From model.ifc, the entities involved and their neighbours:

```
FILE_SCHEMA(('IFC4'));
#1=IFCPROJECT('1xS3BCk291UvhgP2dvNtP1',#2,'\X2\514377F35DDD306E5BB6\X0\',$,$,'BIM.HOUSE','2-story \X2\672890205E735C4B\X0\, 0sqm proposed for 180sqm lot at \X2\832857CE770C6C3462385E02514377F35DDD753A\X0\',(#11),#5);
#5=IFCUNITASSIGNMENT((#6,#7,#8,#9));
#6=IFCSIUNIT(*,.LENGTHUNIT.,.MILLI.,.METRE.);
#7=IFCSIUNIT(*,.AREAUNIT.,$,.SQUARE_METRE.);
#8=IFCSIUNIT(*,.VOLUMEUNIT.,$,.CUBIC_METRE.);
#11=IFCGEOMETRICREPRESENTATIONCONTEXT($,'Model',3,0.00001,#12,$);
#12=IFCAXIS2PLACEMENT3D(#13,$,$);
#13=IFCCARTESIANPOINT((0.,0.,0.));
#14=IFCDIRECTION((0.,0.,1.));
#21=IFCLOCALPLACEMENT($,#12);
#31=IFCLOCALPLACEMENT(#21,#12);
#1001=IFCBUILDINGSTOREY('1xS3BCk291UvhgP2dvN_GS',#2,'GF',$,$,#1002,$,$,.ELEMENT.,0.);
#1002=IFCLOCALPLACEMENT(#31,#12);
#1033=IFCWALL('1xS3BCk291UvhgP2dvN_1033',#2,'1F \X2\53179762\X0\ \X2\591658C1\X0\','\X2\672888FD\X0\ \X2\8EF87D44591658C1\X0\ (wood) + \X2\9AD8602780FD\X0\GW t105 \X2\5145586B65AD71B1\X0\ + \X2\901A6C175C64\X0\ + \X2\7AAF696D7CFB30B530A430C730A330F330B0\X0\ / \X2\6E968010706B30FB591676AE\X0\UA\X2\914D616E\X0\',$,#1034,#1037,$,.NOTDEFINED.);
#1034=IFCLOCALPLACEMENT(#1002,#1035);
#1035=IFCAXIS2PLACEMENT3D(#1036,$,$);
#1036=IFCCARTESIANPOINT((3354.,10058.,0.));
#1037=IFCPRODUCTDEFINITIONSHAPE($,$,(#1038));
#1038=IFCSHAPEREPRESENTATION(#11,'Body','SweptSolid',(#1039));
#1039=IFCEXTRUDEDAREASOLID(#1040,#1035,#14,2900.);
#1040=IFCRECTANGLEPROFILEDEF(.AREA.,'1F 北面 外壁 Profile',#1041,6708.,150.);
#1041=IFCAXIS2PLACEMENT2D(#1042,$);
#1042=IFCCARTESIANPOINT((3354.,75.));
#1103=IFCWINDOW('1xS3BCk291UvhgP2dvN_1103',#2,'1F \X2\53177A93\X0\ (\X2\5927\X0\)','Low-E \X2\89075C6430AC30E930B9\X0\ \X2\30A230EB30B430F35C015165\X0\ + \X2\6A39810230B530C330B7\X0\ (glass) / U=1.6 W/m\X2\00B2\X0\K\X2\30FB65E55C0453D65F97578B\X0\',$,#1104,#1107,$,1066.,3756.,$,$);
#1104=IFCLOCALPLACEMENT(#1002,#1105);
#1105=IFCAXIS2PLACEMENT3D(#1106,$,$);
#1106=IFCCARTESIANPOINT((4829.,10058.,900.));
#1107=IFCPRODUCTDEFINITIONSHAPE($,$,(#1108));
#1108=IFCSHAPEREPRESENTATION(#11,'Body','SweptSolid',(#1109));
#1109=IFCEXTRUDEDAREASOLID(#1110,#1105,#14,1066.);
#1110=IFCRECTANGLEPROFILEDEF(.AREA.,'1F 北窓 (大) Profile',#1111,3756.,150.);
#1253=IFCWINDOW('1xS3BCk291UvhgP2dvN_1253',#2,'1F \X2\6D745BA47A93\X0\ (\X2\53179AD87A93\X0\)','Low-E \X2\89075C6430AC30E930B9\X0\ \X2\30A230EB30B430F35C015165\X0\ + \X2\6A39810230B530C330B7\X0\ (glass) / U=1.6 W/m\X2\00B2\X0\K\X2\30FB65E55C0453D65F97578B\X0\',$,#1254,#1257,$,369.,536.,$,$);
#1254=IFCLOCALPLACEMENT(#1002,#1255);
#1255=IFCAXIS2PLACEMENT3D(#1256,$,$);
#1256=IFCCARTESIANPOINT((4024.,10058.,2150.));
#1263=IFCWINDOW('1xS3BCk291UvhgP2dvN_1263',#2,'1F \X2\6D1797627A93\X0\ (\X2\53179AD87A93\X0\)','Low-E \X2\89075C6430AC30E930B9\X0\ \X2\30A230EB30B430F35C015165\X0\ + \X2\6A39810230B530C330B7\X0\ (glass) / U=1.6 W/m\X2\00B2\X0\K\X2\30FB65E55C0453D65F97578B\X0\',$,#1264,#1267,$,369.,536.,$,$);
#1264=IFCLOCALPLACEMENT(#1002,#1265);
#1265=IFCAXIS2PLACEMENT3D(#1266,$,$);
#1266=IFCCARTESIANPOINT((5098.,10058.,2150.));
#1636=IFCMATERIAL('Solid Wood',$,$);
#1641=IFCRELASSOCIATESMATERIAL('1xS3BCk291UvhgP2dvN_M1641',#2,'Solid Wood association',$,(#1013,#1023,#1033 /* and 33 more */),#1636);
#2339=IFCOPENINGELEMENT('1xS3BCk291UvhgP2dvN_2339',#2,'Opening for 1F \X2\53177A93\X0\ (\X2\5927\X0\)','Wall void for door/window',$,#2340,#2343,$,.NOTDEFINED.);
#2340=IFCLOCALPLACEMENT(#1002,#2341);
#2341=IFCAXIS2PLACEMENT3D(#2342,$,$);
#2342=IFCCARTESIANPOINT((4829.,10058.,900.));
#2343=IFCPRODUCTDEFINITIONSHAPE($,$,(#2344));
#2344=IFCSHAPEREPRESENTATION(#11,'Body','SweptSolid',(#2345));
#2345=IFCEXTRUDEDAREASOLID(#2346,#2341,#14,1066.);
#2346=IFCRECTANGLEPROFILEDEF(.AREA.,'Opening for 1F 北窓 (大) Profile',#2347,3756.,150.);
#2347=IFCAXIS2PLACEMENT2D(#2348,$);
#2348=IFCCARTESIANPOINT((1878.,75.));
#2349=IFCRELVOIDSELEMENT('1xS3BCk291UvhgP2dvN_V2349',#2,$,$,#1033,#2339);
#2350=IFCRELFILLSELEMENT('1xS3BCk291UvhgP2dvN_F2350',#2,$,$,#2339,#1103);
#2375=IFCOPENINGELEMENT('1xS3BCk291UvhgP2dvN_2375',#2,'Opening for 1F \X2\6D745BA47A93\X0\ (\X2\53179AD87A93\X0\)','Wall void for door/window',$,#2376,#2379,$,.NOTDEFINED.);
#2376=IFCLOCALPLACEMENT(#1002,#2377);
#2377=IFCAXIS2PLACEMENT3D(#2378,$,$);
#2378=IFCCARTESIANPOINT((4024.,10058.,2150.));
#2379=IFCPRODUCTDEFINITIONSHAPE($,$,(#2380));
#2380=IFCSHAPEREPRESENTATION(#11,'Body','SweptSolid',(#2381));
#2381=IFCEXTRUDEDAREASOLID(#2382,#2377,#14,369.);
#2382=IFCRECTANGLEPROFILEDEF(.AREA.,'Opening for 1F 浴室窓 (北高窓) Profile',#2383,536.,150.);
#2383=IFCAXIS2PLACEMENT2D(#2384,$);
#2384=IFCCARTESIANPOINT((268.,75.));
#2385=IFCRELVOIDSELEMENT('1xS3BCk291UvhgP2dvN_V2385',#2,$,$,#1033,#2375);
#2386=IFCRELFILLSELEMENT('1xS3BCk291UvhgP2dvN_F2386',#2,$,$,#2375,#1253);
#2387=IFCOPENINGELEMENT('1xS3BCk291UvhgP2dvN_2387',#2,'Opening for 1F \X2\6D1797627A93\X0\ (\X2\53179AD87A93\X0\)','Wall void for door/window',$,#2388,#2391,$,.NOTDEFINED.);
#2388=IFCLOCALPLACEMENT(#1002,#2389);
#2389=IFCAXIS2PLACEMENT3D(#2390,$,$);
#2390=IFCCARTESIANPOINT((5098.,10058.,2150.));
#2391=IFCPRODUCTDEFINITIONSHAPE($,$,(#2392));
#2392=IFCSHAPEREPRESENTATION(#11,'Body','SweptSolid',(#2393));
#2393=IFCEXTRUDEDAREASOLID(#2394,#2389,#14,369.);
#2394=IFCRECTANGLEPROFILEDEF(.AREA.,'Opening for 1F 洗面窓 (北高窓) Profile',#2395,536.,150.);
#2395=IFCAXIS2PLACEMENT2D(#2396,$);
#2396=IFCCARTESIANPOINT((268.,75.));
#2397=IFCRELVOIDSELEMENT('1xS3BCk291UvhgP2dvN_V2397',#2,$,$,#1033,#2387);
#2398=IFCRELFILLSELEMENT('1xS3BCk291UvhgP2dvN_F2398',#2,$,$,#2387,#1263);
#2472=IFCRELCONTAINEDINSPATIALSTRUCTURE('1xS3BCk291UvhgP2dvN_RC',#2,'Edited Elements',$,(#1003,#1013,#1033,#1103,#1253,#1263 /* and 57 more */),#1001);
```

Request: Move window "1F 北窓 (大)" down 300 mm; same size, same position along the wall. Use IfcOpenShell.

```python
import numpy as np
import ifcopenshell
import ifcopenshell.api.geometry
import ifcopenshell.util.placement
import ifcopenshell.util.unit

model = ifcopenshell.open("model.ifc")
unit_scale = ifcopenshell.util.unit.calculate_unit_scale(model)

window = model.by_guid("1xS3BCk291UvhgP2dvN_1103")
opening = window.FillsVoids[0].RelatingOpeningElement
dz = -0.3 / unit_scale

shift = np.array([0.0, 0.0, dz])
# The window is not placed relative to its opening, so move both.
for product in (opening, window):
    matrix = ifcopenshell.util.placement.get_local_placement(product.ObjectPlacement)
    matrix[:3, 3] += shift
    ifcopenshell.api.geometry.edit_object_placement(model, product=product, matrix=matrix, is_si=False)

print(f"moved by {dz * unit_scale:+.3f} m")

model.write("model-out.ifc")
```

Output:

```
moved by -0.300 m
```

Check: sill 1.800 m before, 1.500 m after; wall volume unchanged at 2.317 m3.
